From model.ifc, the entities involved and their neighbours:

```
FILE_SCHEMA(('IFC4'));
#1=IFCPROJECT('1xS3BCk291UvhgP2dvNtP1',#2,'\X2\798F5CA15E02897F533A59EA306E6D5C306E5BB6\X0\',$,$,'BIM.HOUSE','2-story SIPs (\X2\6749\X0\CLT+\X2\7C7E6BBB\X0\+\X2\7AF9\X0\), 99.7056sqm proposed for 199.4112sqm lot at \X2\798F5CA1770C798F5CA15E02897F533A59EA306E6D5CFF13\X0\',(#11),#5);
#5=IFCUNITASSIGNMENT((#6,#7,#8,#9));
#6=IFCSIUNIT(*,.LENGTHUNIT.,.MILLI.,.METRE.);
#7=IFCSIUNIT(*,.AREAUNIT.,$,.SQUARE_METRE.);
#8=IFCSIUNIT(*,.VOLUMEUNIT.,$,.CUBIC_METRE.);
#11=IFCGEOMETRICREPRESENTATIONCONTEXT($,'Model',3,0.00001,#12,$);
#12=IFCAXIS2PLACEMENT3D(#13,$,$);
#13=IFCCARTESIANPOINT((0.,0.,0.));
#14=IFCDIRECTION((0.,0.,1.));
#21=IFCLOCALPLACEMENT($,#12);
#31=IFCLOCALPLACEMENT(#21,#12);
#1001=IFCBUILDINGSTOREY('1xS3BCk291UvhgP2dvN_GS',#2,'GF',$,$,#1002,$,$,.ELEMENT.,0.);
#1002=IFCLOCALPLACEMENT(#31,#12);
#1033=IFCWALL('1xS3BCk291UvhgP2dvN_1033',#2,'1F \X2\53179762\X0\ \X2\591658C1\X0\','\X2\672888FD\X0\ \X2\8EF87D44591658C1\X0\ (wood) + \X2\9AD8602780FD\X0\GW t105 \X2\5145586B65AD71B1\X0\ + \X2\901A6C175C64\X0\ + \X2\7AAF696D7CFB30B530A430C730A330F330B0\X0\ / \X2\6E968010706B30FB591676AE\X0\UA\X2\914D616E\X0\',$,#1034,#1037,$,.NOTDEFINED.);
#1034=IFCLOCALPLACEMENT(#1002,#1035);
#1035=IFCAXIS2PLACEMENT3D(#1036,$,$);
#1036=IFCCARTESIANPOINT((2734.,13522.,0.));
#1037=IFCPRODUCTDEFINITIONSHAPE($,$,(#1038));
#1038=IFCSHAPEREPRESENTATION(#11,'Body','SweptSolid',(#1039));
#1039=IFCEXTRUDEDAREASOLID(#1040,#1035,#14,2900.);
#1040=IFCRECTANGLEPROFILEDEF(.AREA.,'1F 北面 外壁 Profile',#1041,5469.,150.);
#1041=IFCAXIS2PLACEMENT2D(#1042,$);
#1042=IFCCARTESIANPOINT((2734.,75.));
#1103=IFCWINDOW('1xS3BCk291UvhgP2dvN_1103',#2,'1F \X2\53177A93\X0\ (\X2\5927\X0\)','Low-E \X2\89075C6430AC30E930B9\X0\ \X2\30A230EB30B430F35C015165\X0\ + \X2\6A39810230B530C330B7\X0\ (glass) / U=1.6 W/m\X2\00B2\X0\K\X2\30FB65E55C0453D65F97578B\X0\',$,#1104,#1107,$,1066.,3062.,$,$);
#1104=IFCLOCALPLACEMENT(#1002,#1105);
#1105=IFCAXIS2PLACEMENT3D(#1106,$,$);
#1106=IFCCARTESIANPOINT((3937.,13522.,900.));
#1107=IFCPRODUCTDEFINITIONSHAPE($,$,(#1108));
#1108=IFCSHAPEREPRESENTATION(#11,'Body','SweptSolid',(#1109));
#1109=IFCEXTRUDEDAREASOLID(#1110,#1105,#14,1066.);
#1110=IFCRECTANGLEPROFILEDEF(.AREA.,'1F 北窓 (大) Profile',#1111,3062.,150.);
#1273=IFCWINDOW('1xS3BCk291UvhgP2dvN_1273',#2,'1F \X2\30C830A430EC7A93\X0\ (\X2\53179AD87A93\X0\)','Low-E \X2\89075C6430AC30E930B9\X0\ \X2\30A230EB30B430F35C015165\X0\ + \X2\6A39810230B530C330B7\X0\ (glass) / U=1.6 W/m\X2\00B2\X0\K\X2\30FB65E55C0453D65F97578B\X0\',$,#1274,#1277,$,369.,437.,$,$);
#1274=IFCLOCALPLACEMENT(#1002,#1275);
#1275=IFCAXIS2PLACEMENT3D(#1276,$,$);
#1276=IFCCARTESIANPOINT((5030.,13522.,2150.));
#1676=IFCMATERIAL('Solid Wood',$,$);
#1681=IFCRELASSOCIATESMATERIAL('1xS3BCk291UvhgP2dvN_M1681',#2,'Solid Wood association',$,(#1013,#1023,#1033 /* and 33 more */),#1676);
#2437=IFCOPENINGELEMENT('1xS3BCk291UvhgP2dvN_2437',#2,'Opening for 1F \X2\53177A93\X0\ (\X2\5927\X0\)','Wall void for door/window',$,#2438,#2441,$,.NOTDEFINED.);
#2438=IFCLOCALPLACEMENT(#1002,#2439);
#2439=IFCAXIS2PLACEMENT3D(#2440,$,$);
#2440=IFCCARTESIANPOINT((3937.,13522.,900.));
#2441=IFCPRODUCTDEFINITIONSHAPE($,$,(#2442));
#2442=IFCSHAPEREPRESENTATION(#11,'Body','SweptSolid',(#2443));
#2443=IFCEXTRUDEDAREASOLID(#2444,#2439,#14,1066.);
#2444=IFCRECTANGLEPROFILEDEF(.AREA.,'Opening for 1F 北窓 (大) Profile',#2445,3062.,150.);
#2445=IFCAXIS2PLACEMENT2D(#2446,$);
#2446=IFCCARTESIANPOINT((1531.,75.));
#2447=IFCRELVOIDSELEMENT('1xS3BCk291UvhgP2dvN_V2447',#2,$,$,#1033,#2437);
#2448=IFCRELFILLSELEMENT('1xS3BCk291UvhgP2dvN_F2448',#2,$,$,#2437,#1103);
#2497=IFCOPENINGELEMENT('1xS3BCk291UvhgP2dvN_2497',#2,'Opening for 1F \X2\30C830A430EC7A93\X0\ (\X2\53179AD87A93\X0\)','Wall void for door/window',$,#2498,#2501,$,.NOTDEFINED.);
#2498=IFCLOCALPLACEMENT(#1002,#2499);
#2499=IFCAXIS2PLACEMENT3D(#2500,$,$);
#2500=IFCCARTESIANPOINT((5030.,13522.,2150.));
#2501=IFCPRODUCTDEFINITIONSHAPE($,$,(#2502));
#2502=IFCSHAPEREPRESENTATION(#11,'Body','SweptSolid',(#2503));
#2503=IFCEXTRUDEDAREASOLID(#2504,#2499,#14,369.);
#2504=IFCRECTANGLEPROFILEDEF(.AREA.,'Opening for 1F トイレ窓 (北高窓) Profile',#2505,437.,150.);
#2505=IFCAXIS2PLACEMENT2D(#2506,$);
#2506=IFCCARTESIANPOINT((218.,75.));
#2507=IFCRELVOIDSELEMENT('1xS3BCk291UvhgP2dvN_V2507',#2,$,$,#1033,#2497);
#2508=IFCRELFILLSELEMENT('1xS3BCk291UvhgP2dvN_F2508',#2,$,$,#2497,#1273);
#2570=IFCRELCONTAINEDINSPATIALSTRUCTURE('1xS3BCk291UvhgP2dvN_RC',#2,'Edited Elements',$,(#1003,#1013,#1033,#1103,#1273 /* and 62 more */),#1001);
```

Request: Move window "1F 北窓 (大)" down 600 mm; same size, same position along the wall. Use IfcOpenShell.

```python
import numpy as np
import ifcopenshell
import ifcopenshell.api.geometry
import ifcopenshell.util.placement
import ifcopenshell.util.unit

model = ifcopenshell.open("model.ifc")
unit_scale = ifcopenshell.util.unit.calculate_unit_scale(model)

window = model.by_guid("1xS3BCk291UvhgP2dvN_1103")
opening = window.FillsVoids[0].RelatingOpeningElement
dz = -600.0

shift = np.array([0.0, 0.0, dz])
# The window is not placed relative to its opening, so move both.
for product in (opening, window):
    matrix = ifcopenshell.util.placement.get_local_placement(product.ObjectPlacement)
    matrix[:3, 3] += shift
    ifcopenshell.api.geometry.edit_object_placement(model, product=product, matrix=matrix, is_si=False)

print(f"moved by {dz * unit_scale:+.3f} m")

model.write("model_v2.ifc")
```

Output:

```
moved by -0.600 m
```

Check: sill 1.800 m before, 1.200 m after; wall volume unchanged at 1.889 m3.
